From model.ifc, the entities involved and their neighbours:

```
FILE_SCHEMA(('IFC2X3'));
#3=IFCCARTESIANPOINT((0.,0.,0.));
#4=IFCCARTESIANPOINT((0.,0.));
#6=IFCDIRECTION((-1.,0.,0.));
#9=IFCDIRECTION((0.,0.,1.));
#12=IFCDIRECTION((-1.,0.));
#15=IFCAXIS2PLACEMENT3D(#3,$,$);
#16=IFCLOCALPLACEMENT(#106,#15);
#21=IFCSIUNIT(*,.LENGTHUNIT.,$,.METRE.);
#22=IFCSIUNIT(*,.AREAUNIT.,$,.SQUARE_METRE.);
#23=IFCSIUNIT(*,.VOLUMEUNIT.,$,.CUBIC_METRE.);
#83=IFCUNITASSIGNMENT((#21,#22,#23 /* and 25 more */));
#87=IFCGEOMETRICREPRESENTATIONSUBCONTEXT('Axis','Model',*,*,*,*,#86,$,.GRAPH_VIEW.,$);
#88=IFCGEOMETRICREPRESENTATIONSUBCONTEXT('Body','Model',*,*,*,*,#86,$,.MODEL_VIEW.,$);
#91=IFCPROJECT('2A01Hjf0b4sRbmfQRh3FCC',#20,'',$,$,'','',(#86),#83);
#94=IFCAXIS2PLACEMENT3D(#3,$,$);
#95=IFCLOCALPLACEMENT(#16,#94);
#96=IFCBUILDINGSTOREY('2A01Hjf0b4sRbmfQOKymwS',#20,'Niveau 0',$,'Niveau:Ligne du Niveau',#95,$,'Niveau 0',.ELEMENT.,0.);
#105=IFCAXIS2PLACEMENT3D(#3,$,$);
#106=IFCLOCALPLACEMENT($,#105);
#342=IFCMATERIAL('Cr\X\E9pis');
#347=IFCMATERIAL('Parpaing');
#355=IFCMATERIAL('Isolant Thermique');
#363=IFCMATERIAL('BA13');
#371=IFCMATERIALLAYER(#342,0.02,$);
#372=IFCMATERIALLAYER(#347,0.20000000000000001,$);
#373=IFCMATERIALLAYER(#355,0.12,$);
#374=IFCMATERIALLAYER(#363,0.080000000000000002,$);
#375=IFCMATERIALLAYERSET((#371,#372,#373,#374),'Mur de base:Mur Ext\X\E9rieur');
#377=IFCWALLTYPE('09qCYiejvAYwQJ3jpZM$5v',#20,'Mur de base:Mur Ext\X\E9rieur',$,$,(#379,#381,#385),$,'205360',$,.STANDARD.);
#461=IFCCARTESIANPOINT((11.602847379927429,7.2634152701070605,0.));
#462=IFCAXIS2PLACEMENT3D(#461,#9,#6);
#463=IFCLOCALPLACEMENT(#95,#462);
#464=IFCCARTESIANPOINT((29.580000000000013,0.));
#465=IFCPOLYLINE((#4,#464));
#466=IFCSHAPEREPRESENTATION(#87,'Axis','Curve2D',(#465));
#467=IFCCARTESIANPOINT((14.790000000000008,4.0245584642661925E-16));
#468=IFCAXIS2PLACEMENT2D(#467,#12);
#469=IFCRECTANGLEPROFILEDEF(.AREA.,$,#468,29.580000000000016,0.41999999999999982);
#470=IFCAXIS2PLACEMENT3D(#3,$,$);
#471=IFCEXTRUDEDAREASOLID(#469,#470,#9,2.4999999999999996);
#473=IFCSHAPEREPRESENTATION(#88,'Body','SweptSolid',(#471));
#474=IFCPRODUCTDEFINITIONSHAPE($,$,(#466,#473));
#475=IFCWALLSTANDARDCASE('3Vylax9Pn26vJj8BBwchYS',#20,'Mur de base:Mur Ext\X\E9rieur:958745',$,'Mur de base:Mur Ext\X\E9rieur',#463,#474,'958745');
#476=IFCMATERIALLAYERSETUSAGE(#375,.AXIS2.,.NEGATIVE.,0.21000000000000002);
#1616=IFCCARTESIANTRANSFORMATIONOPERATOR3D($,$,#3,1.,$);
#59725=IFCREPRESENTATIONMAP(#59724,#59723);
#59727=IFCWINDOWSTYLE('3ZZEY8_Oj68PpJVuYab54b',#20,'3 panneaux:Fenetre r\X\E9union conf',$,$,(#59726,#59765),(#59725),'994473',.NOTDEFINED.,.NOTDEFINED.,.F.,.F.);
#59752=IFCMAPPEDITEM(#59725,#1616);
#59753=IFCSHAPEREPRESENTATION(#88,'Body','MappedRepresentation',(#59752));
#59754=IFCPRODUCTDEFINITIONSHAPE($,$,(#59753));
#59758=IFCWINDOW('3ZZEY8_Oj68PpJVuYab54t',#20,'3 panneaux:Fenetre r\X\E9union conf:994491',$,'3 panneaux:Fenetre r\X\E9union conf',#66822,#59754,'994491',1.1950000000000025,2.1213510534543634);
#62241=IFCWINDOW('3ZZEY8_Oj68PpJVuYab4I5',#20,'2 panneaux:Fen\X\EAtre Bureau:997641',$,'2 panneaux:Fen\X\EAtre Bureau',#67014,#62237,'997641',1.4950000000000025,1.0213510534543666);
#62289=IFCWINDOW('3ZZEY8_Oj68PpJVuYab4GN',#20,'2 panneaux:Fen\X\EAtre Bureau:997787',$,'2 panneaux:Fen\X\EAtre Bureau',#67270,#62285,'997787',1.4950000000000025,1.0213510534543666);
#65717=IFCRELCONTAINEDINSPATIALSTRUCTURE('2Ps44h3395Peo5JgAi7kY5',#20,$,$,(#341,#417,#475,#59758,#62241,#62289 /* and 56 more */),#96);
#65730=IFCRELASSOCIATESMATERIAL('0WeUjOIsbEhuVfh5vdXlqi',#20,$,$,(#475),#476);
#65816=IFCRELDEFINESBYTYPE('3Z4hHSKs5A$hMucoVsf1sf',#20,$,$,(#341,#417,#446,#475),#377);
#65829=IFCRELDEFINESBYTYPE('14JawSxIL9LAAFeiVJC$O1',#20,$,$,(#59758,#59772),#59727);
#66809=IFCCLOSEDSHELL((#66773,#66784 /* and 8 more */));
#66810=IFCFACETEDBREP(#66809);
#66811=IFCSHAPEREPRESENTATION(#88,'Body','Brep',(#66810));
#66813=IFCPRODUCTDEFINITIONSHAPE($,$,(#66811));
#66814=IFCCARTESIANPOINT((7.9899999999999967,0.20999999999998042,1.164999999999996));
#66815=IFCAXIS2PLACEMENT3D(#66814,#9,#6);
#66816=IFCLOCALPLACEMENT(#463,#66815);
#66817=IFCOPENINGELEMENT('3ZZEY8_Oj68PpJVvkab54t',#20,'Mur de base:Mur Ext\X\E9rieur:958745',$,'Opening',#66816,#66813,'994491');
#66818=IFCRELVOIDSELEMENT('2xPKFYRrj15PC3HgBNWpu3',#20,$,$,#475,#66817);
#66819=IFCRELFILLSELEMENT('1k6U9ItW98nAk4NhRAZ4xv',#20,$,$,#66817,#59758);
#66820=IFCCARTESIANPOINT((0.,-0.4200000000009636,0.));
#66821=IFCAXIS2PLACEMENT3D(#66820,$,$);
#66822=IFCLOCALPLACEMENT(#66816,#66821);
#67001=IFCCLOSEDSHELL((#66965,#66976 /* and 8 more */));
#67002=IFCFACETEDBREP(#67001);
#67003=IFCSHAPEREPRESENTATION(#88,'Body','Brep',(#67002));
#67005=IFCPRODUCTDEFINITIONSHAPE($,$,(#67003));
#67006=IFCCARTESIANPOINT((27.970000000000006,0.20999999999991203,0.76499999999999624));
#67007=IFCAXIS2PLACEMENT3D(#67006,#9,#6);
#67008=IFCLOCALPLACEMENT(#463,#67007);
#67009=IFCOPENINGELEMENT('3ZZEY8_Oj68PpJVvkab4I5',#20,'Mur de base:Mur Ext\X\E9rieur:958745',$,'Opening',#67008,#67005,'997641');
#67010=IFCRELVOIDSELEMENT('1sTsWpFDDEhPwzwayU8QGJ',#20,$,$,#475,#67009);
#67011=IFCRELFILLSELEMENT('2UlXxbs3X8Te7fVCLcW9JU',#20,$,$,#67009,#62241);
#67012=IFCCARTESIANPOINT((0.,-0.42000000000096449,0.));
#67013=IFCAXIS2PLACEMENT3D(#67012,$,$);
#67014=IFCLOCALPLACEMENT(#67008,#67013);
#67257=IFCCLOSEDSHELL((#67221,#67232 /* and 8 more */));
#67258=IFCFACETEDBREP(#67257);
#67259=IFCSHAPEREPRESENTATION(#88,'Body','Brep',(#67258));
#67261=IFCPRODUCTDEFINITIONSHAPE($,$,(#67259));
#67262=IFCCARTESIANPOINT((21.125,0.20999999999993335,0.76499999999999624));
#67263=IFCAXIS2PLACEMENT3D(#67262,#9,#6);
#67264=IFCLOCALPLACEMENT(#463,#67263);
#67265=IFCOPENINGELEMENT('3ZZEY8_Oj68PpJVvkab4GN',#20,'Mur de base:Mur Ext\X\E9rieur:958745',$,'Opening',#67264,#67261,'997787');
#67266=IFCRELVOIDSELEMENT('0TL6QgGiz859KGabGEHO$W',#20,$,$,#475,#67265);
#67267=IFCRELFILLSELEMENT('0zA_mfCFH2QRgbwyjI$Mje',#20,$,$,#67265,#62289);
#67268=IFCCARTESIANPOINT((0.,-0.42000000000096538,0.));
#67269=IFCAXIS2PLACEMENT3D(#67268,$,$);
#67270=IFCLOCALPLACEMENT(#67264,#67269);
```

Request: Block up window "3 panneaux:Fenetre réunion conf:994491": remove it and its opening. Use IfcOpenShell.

```python
import ifcopenshell
import ifcopenshell.api.feature
import ifcopenshell.api.root
import ifcopenshell.geom
import ifcopenshell.util.shape

model = ifcopenshell.open("model.ifc")
settings = ifcopenshell.geom.settings()


def volume(element):
    """Net volume in cubic metres, openings subtracted."""
    shape = ifcopenshell.geom.create_shape(settings, element)
    return ifcopenshell.util.shape.get_volume(shape.geometry)


window = model.by_id(59758)
opening = window.FillsVoids[0].RelatingOpeningElement
wall = opening.VoidsElements[0].RelatingBuildingElement
before = volume(wall)

ifcopenshell.api.root.remove_product(model, product=window)
ifcopenshell.api.feature.remove_feature(model, feature=opening)

after = volume(wall)

print(f"wall volume {before:.3f} -> {after:.3f} m3")

model.write("model_v2.ifc")
```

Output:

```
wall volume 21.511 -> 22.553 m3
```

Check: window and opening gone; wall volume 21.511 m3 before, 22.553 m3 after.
